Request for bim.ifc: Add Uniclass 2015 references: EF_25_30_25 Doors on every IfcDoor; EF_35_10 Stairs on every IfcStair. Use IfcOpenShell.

First a look at what the model holds.

```python
import ifcopenshell

model = ifcopenshell.open("bim.ifc")
print(model.schema)
print("classifications:", [c.Name for c in model.by_type("IfcClassification")])
for ifc_class in ("IfcDoor", "IfcRoof", "IfcStair", "IfcWall", "IfcWindow"):
    print(ifc_class, len(model.by_type(ifc_class)))
```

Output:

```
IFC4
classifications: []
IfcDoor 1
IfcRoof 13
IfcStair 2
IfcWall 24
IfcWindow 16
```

```python
import ifcopenshell
import ifcopenshell.api.classification

model = ifcopenshell.open("bim.ifc")

system = ifcopenshell.api.classification.add_classification(model, classification="Uniclass 2015")

codes = {
    "IfcDoor": ("EF_25_30_25", "Doors"),
    "IfcStair": ("EF_35_10", "Stairs"),
}
for ifc_class, (code, name) in codes.items():
    products = model.by_type(ifc_class)
    ifcopenshell.api.classification.add_reference(
        model, products=products, classification=system, identification=code, name=name
    )
    print(code, len(products))

model.write("bim-out.ifc")
```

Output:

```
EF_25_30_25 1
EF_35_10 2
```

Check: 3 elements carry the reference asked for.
